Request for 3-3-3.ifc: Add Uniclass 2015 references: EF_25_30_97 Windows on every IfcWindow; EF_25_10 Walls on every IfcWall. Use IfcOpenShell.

First a look at what the model holds.

```python
import ifcopenshell

model = ifcopenshell.open("3-3-3.ifc")
print(model.schema)
print("classifications:", [c.Name for c in model.by_type("IfcClassification")])
for ifc_class in ("IfcDoor", "IfcRoof", "IfcStair", "IfcWall", "IfcWindow"):
    print(ifc_class, len(model.by_type(ifc_class)))
```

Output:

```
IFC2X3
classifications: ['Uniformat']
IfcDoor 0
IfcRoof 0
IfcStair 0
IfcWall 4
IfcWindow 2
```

```python
import ifcopenshell
import ifcopenshell.api.classification

model = ifcopenshell.open("3-3-3.ifc")

# IFC2X3 requires Source and Edition and has no link from the project to the system.
system = model.create_entity("IfcClassification", Source="NBS", Edition="2015", Name="Uniclass 2015")

codes = {
    "IfcWindow": ("EF_25_30_97", "Windows"),
    "IfcWall": ("EF_25_10", "Walls"),
}
for ifc_class, (code, name) in codes.items():
    products = model.by_type(ifc_class)
    ifcopenshell.api.classification.add_reference(
        model, products=products, classification=system, identification=code, name=name
    )
    print(code, len(products))

model.write("3-3-3-out.ifc")
```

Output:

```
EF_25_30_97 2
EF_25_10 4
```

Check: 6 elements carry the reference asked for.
